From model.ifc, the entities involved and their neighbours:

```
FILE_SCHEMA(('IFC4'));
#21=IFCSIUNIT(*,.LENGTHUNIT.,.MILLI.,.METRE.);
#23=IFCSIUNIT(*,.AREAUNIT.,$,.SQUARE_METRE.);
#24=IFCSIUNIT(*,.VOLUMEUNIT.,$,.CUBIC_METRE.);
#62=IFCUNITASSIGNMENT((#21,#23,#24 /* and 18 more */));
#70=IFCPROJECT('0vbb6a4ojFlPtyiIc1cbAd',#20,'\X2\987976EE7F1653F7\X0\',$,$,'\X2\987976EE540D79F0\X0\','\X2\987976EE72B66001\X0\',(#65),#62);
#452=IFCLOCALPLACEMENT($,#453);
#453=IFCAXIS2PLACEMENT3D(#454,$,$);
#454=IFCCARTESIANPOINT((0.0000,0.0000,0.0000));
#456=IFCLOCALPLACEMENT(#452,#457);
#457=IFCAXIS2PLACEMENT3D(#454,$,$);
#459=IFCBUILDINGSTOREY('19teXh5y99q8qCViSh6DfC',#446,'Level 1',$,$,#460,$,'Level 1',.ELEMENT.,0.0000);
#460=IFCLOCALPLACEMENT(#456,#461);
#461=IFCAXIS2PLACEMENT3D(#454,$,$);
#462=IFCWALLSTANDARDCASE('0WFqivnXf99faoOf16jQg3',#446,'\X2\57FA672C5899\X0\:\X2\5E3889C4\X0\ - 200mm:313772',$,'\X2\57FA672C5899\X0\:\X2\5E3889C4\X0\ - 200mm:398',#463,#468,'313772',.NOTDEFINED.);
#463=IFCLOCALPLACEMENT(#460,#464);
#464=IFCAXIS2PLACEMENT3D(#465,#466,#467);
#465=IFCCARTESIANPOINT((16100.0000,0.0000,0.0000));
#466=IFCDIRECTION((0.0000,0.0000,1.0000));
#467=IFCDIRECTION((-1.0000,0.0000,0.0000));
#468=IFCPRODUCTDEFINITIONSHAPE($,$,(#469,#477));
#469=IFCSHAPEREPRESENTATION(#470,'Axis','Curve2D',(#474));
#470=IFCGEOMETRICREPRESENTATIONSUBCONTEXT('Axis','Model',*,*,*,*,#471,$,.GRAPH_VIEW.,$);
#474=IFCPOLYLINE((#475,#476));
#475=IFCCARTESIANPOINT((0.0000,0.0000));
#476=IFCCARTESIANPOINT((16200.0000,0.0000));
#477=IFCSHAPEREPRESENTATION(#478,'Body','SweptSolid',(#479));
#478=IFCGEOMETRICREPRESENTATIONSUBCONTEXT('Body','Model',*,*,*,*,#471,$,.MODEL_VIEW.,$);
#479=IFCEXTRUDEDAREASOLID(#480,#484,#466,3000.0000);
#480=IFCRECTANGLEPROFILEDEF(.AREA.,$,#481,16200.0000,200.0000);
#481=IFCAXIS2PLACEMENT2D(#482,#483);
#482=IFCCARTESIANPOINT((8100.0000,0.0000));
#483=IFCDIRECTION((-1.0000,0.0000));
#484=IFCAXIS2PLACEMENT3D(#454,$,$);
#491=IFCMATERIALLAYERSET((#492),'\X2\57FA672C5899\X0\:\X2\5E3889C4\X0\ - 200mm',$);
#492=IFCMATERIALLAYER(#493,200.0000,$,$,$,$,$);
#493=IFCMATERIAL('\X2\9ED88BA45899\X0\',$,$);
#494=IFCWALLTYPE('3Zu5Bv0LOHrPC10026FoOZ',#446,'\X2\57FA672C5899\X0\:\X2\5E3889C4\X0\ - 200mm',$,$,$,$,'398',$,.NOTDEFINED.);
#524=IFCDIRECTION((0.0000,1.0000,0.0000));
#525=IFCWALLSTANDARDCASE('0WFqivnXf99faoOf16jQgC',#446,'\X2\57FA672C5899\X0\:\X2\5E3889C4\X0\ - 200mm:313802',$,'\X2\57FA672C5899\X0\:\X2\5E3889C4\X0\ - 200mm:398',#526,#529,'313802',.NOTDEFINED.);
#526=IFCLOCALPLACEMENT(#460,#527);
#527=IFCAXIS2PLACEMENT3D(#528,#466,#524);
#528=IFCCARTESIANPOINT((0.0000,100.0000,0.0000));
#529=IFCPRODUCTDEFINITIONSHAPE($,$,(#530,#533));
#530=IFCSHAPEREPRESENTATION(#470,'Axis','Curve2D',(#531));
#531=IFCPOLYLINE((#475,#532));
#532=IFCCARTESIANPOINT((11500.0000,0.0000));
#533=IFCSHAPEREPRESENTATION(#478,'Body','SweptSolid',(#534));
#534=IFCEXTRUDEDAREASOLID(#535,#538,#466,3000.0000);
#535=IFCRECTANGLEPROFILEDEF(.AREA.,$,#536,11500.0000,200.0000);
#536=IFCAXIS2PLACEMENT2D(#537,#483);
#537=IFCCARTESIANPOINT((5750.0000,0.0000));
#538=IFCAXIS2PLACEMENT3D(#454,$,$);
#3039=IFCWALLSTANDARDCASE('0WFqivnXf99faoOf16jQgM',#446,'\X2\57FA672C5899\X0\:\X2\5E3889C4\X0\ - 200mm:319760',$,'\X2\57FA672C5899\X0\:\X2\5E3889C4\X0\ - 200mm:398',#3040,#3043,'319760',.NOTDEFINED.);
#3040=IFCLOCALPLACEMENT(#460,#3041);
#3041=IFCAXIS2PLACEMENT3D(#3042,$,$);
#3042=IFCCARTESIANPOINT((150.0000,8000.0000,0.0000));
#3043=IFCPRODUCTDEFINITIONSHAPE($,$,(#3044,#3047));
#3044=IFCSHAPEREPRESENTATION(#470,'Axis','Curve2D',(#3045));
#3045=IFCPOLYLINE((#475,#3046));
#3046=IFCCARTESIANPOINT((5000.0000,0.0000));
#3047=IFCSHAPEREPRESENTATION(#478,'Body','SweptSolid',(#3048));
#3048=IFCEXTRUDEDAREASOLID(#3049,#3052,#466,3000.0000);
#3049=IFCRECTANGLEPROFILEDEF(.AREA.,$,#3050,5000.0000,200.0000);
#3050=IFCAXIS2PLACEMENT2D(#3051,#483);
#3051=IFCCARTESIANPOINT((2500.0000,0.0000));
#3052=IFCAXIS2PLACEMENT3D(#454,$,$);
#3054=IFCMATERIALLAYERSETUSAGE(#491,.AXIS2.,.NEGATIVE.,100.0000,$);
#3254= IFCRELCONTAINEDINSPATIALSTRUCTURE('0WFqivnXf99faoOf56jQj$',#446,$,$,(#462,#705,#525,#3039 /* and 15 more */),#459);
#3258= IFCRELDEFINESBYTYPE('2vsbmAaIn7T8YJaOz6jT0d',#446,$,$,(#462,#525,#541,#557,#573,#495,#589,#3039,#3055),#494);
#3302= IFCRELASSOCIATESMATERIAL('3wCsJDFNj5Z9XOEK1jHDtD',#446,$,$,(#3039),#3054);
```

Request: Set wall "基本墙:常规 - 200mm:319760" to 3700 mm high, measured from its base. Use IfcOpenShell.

```python
import ifcopenshell
import ifcopenshell.geom
import ifcopenshell.util.representation
import ifcopenshell.util.shape

model = ifcopenshell.open("model.ifc")
settings = ifcopenshell.geom.settings()


def volume(element):
    """Net volume in cubic metres, openings subtracted."""
    shape = ifcopenshell.geom.create_shape(settings, element)
    return ifcopenshell.util.shape.get_volume(shape.geometry)


wall = model.by_guid("0WFqivnXf99faoOf16jQgM")
before = volume(wall)

body = ifcopenshell.util.representation.get_representation(wall, "Model", "Body")
solid = body.Items[0]
old_height = solid.Depth
solid.Depth = 3700.0
after = volume(wall)

print(f"height {old_height:g} -> {solid.Depth:g}, volume {before:.3f} -> {after:.3f} m3")

model.write("model_rev.ifc")
```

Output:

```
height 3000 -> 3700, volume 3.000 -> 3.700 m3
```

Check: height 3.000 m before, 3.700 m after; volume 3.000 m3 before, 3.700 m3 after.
